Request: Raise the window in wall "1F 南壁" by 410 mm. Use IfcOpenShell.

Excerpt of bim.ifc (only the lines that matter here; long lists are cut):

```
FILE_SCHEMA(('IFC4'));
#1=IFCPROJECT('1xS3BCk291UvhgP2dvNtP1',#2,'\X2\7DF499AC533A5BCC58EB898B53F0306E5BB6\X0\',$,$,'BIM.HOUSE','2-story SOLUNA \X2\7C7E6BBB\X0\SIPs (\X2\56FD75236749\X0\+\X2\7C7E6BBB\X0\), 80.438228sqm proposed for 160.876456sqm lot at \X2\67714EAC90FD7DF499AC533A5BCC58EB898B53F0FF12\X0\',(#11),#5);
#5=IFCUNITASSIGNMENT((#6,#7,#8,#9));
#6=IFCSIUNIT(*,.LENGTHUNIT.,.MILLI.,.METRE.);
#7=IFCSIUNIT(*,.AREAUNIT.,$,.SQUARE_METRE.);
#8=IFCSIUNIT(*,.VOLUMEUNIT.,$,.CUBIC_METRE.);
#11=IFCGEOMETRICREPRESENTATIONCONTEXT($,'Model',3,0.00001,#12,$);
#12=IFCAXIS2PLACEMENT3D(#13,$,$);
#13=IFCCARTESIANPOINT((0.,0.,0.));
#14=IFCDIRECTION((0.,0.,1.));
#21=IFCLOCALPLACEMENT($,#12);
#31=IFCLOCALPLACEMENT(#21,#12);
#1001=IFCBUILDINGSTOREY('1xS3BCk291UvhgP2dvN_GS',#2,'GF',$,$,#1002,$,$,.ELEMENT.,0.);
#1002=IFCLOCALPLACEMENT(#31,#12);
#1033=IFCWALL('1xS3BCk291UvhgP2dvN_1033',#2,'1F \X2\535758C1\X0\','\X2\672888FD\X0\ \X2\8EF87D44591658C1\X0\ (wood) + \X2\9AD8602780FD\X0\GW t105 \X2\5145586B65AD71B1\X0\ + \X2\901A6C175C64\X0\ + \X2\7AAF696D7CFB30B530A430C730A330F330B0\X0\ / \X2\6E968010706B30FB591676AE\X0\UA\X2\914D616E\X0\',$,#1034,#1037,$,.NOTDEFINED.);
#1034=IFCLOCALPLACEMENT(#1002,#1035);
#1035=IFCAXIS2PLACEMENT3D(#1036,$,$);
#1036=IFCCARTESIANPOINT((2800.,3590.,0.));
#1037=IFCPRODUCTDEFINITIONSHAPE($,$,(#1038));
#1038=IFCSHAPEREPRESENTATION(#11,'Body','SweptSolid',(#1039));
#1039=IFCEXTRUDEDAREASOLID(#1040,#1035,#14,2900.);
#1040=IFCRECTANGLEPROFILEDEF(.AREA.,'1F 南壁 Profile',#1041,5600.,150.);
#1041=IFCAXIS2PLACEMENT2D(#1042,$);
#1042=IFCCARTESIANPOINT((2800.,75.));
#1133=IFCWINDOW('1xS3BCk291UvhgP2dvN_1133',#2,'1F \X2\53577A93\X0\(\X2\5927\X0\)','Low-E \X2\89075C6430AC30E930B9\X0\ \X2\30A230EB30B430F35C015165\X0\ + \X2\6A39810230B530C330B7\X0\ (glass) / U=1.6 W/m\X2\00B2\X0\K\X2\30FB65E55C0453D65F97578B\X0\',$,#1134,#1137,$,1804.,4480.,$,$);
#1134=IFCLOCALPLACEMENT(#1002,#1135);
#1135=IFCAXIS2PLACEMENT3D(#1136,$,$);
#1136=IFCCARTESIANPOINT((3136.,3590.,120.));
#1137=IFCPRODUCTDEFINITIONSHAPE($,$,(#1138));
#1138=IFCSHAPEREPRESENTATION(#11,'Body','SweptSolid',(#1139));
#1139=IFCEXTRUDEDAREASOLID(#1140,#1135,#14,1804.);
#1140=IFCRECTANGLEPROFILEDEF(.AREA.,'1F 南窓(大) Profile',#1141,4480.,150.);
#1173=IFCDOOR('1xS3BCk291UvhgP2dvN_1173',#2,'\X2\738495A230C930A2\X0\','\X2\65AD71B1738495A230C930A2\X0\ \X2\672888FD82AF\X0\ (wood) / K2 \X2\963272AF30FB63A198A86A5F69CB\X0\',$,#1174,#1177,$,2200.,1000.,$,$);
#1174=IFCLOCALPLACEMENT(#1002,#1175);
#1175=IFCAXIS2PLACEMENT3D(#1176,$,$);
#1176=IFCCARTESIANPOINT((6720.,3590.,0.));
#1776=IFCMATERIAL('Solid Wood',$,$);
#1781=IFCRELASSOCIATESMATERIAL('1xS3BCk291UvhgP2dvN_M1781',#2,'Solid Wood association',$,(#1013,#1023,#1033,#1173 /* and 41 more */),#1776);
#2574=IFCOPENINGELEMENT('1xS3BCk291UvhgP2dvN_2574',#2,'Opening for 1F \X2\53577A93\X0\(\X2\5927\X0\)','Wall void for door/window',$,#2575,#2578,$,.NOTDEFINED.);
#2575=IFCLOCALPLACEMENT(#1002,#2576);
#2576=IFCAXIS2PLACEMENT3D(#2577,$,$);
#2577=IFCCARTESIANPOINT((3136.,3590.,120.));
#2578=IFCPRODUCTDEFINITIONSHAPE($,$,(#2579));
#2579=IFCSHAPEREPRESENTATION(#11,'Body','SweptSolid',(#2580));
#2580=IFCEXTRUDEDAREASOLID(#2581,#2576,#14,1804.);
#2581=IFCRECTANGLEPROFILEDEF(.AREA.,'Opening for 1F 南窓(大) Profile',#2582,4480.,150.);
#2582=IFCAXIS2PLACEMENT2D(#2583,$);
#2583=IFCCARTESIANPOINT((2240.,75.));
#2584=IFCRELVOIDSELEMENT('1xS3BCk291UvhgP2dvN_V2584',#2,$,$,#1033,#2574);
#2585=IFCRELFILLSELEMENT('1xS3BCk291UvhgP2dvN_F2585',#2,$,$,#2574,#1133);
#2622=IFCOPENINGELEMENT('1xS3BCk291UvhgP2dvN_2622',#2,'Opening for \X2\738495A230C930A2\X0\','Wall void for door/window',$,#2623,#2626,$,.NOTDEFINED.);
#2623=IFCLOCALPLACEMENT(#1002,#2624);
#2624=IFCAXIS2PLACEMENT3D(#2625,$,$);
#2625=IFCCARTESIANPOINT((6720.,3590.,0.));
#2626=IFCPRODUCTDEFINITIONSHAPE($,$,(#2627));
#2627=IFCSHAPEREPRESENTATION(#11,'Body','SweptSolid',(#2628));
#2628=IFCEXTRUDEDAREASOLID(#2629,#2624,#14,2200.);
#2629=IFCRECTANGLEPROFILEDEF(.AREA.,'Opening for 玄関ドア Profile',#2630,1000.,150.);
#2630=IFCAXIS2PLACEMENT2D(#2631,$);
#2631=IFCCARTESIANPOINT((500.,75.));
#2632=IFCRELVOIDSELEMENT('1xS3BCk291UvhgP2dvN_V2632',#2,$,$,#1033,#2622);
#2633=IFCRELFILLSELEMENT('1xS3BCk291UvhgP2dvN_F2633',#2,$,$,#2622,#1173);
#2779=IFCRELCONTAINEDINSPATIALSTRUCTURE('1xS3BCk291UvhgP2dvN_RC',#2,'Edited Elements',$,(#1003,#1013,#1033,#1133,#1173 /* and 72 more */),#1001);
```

```python
import numpy as np
import ifcopenshell
import ifcopenshell.api.geometry
import ifcopenshell.util.placement
import ifcopenshell.util.unit

model = ifcopenshell.open("bim.ifc")
unit_scale = ifcopenshell.util.unit.calculate_unit_scale(model)

window = model.by_guid("1xS3BCk291UvhgP2dvN_1133")
opening = window.FillsVoids[0].RelatingOpeningElement
dz = 0.41 / unit_scale

shift = np.array([0.0, 0.0, dz])
# The window is not placed relative to its opening, so move both.
for product in (opening, window):
    matrix = ifcopenshell.util.placement.get_local_placement(product.ObjectPlacement)
    matrix[:3, 3] += shift
    ifcopenshell.api.geometry.edit_object_placement(model, product=product, matrix=matrix, is_si=False)

print(f"moved by {dz * unit_scale:+.3f} m")

model.write("bim_rev.ifc")
```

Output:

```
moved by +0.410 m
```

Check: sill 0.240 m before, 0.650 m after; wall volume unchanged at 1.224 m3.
